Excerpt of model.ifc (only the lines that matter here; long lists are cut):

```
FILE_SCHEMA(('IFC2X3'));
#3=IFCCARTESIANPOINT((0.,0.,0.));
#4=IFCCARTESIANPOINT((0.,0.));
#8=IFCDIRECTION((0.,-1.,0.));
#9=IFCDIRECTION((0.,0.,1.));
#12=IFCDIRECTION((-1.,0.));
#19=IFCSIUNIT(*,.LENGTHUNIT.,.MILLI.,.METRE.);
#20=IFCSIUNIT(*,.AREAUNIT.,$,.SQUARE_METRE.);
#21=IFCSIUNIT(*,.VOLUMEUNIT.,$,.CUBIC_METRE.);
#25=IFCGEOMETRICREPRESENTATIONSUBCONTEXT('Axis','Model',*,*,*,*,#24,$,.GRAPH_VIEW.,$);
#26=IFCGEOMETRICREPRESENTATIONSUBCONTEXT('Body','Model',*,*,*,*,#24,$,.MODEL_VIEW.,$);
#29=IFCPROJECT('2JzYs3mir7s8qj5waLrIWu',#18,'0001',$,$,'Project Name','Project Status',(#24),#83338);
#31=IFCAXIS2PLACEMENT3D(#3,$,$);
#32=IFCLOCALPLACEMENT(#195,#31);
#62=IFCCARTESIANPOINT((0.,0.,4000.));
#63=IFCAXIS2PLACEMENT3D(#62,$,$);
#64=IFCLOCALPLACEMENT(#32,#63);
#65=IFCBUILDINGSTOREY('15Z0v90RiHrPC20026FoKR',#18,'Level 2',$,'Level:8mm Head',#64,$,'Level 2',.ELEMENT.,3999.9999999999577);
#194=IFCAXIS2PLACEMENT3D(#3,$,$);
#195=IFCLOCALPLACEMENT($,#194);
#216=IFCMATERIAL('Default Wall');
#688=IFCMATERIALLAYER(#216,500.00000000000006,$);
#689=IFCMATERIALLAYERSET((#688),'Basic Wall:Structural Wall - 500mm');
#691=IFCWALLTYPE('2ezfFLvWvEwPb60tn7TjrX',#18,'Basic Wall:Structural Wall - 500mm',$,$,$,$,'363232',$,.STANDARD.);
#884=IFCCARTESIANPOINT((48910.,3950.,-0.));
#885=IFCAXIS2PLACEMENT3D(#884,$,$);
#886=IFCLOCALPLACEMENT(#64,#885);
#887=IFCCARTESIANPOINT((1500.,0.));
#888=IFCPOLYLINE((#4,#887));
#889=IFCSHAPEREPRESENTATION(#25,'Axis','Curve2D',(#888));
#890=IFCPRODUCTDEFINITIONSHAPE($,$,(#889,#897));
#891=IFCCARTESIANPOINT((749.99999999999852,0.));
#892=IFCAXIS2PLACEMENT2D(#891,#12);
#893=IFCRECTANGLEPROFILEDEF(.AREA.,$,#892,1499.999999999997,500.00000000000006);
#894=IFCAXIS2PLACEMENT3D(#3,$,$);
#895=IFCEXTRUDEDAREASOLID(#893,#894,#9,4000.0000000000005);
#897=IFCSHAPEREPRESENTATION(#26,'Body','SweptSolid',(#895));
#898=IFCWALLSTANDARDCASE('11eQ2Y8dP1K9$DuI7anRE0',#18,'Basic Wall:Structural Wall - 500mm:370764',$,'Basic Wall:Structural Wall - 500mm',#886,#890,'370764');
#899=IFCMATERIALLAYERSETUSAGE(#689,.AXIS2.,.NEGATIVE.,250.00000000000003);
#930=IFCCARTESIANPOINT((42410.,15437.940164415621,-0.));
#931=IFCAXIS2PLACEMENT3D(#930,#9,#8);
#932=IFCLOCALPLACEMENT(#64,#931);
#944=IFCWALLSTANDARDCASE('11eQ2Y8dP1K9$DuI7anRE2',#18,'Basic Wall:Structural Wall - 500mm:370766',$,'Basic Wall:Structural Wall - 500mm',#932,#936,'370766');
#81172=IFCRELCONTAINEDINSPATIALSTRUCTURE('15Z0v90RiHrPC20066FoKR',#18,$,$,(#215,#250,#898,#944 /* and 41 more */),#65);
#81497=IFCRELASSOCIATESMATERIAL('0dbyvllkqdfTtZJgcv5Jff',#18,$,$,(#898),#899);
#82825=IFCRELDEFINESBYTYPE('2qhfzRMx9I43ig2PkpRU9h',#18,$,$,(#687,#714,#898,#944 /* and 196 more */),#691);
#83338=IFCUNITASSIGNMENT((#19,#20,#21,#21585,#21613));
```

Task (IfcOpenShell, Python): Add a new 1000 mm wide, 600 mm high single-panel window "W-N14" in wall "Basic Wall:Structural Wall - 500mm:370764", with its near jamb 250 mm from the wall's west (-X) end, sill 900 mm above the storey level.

```python
import numpy as np
import ifcopenshell
import ifcopenshell.api.feature
import ifcopenshell.api.geometry
import ifcopenshell.api.root
import ifcopenshell.api.spatial
import ifcopenshell.api.type
import ifcopenshell.geom
import ifcopenshell.util.element
import ifcopenshell.util.placement
import ifcopenshell.util.representation
import ifcopenshell.util.shape
import ifcopenshell.util.unit

model = ifcopenshell.open("model.ifc")
unit_scale = ifcopenshell.util.unit.calculate_unit_scale(model)
settings = ifcopenshell.geom.settings()


def volume(element):
    """Net volume in cubic metres, openings subtracted."""
    shape = ifcopenshell.geom.create_shape(settings, element)
    return ifcopenshell.util.shape.get_volume(shape.geometry)


wall = model.by_guid("11eQ2Y8dP1K9$DuI7anRE0")
storey = ifcopenshell.util.element.get_container(wall, ifc_class="IfcBuildingStorey")
context = ifcopenshell.util.representation.get_context(model, "Model", "Body", "MODEL_VIEW")
before = volume(wall)

width, height, from_end, sill = 1, 0.6, 0.25, 0.9  # metres

# The wall runs along its own X axis, and the end named is its -X end.
wall_shape = ifcopenshell.geom.create_shape(settings, wall)
x, y, z = ifcopenshell.util.shape.get_vertices(wall_shape.geometry).T
start = x.min() + from_end
face, thickness = float(y.min()), float(y.max() - y.min())
wall_matrix = ifcopenshell.util.placement.get_local_placement(wall.ObjectPlacement)
level = ifcopenshell.util.placement.get_local_placement(storey.ObjectPlacement)[2, 3]


def in_wall(x, y):
    """Placement at x, y metres in the wall's axes, at sill height."""
    matrix = wall_matrix.copy()
    matrix[:, 3] = wall_matrix @ np.array([x / unit_scale, y / unit_scale, 0.0, 1.0])
    matrix[2, 3] = level + sill / unit_scale
    return matrix


# Opening: a box that overshoots both wall faces by 50 mm.
opening = ifcopenshell.api.root.create_entity(model, ifc_class="IfcOpeningElement")
box = ifcopenshell.api.geometry.add_wall_representation(
    model, context=context, length=width, height=height, thickness=thickness + 0.1
)
ifcopenshell.api.geometry.assign_representation(model, product=opening, representation=box)
ifcopenshell.api.geometry.edit_object_placement(model, product=opening, matrix=in_wall(start, face - 0.05), is_si=False)
ifcopenshell.api.feature.add_feature(model, feature=opening, element=wall)

window = ifcopenshell.api.root.create_entity(model, ifc_class="IfcWindow", name="W-N14")
window.OverallWidth, window.OverallHeight = width / unit_scale, height / unit_scale
body = ifcopenshell.api.geometry.add_window_representation(
    model,
    context=context,
    overall_width=window.OverallWidth,
    overall_height=window.OverallHeight,
    partition_type="SINGLE_PANEL",
)
ifcopenshell.api.geometry.assign_representation(model, product=window, representation=body)
ifcopenshell.api.spatial.assign_container(model, products=[window], relating_structure=storey)
fills = ifcopenshell.api.feature.add_filling(model, opening=opening, element=window)
fills.OwnerHistory = window.OwnerHistory  # required in IFC2X3

# IFC2X3 keeps the operation on the window style.
style = ifcopenshell.api.root.create_entity(model, ifc_class="IfcWindowStyle", name="W-N14")
style.OperationType, style.ConstructionType = "SINGLE_PANEL", "NOTDEFINED"
style.ParameterTakesPrecedence = style.Sizeable = False
ifcopenshell.api.type.assign_type(model, related_objects=[window], relating_type=style)

# Centre the window in the wall's thickness.
ifcopenshell.api.geometry.edit_object_placement(model, product=window, matrix=in_wall(start, face), is_si=False)
window_shape = ifcopenshell.geom.create_shape(settings, window)
depth = ifcopenshell.util.shape.get_vertices(window_shape.geometry)[:, 1]
offset = face + thickness / 2 - (depth.min() + depth.max()) / 2
ifcopenshell.api.geometry.edit_object_placement(model, product=window, matrix=in_wall(start, offset), is_si=False)

after = volume(wall)

print(f"wall volume {before:.3f} -> {after:.3f} m3")

model.write("model_updated.ifc")
```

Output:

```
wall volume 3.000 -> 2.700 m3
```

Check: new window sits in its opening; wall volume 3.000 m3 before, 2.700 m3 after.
